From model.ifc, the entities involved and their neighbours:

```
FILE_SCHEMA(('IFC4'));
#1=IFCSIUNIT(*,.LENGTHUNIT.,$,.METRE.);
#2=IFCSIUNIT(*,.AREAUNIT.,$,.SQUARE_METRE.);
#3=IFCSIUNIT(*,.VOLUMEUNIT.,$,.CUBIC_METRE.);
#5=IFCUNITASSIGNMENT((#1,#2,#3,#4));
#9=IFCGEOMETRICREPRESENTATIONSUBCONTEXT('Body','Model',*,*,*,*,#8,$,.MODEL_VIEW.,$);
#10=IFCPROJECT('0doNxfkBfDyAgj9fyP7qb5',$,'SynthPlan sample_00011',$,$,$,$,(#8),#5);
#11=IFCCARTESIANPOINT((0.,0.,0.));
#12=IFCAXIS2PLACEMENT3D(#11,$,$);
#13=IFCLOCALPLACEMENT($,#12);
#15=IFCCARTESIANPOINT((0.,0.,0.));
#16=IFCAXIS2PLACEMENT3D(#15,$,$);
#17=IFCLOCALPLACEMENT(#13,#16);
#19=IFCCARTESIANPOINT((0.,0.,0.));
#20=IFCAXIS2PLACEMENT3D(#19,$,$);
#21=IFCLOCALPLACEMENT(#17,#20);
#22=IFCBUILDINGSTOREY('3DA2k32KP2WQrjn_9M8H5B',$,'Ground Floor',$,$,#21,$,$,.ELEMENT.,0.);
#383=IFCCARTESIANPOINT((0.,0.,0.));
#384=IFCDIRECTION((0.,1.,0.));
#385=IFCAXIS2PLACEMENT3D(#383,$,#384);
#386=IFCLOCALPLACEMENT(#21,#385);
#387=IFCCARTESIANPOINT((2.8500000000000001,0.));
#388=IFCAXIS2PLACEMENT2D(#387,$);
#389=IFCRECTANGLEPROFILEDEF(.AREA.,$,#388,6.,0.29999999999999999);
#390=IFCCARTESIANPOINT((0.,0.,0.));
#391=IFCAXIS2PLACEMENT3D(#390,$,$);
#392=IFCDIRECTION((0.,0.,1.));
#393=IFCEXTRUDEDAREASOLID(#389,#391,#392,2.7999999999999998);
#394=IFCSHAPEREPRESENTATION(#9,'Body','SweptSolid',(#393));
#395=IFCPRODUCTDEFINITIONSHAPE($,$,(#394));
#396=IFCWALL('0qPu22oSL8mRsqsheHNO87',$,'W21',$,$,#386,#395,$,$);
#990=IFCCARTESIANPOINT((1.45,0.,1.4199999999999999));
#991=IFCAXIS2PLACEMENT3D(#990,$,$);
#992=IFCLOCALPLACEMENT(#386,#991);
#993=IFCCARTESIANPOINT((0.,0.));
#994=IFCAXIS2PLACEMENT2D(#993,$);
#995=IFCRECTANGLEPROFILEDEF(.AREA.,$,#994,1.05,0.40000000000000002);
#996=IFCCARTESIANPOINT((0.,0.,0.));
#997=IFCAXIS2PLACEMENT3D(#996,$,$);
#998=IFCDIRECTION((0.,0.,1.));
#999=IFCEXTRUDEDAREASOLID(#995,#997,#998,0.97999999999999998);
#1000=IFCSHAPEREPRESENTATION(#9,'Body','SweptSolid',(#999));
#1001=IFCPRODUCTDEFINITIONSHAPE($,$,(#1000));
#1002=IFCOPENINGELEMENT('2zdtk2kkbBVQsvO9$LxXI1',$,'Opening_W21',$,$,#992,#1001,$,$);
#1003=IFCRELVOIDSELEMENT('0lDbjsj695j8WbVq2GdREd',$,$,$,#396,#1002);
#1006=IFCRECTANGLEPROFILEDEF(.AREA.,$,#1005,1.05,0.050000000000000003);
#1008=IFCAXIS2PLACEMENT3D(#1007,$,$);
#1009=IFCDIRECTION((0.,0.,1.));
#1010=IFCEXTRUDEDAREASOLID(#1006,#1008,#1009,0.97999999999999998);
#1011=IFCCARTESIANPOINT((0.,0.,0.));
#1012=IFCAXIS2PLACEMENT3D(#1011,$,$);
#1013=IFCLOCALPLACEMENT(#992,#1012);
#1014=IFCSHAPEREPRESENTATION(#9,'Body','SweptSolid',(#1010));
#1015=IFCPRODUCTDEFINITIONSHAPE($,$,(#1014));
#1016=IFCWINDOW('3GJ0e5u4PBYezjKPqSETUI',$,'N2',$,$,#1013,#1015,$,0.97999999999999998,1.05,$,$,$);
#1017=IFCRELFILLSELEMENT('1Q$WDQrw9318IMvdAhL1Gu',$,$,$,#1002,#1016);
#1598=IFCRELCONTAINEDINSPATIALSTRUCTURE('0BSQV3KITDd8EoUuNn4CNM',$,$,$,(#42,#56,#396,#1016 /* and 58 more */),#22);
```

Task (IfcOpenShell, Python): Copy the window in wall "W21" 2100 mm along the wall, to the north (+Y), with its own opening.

```python
import ifcopenshell
import ifcopenshell.api.feature
import ifcopenshell.api.geometry
import ifcopenshell.api.root
import ifcopenshell.geom
import ifcopenshell.util.element
import ifcopenshell.util.placement
import ifcopenshell.util.shape
import ifcopenshell.util.unit

model = ifcopenshell.open("model.ifc")
unit_scale = ifcopenshell.util.unit.calculate_unit_scale(model)
settings = ifcopenshell.geom.settings()


def volume(element):
    """Net volume in cubic metres, openings subtracted."""
    shape = ifcopenshell.geom.create_shape(settings, element)
    return ifcopenshell.util.shape.get_volume(shape.geometry)


window = model.by_guid("3GJ0e5u4PBYezjKPqSETUI")
opening = window.FillsVoids[0].RelatingOpeningElement
wall = opening.VoidsElements[0].RelatingBuildingElement
before = volume(wall)
shift = ifcopenshell.util.placement.get_local_placement(wall.ObjectPlacement)[:3, 0] * 2.1 / unit_scale

# copy_class copies the void relationship, type, container and properties, but no geometry.
new_opening = ifcopenshell.api.root.copy_class(model, product=opening)
new_opening.Representation = ifcopenshell.util.element.copy_deep(
    model, opening.Representation, exclude=["IfcGeometricRepresentationContext", "IfcRepresentationMap"]
)
new_window = ifcopenshell.api.root.copy_class(model, product=window)
new_window.Representation = ifcopenshell.util.element.copy_deep(
    model, window.Representation, exclude=["IfcGeometricRepresentationContext", "IfcRepresentationMap"]
)
ifcopenshell.api.feature.add_filling(model, opening=new_opening, element=new_window)

for old, new in ((opening, new_opening), (window, new_window)):
    matrix = ifcopenshell.util.placement.get_local_placement(old.ObjectPlacement)
    matrix[:3, 3] += shift
    ifcopenshell.api.geometry.edit_object_placement(model, product=new, matrix=matrix, is_si=False)

after = volume(wall)

print(f"wall volume {before:.3f} -> {after:.3f} m3")

model.write("model-out.ifc")
```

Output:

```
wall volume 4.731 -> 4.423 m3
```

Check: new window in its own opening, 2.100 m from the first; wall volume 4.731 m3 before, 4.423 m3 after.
